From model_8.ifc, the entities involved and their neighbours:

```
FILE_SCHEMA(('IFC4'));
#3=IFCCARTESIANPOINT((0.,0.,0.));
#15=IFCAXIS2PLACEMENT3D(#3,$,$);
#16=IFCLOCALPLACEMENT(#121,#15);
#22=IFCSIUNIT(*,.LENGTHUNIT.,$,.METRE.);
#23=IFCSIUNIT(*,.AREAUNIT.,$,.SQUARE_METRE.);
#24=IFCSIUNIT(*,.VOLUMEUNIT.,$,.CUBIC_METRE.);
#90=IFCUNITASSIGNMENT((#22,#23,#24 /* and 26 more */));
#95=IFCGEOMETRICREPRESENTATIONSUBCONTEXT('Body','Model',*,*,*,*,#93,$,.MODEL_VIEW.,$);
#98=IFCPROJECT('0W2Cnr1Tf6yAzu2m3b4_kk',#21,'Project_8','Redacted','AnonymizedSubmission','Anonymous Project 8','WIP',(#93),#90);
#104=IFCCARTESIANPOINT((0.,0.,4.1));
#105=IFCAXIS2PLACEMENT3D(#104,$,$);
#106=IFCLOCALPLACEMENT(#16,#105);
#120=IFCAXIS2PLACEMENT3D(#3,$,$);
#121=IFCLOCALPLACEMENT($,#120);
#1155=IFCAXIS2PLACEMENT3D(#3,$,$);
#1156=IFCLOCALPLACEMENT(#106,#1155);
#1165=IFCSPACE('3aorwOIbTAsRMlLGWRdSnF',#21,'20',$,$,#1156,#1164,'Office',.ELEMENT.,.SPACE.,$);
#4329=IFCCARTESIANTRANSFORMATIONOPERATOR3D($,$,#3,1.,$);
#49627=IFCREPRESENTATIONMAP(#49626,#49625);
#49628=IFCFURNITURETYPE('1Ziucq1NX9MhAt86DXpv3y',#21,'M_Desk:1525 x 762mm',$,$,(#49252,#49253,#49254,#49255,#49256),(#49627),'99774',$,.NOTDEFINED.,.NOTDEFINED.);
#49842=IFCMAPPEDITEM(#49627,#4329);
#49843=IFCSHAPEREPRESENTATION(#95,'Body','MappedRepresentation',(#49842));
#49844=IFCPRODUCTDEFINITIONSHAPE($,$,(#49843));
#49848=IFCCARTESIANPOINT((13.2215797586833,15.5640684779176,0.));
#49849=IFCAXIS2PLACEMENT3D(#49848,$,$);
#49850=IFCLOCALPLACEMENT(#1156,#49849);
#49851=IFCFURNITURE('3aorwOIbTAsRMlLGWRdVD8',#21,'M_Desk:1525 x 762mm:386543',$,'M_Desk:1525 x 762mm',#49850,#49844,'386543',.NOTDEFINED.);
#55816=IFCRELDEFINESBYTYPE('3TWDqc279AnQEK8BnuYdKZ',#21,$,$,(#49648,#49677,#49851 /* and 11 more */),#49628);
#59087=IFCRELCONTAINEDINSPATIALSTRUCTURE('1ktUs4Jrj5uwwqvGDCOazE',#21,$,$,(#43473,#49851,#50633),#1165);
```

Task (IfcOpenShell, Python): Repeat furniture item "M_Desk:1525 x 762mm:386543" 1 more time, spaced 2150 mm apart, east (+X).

```python
import numpy as np
import ifcopenshell
import ifcopenshell.api.geometry
import ifcopenshell.api.root
import ifcopenshell.util.element
import ifcopenshell.util.placement
import ifcopenshell.util.unit

model = ifcopenshell.open("model_8.ifc")
unit_scale = ifcopenshell.util.unit.calculate_unit_scale(model)


def reuse_history(source, copy):
    """copy_class also copies each property set's owner history, people and application; keep the originals."""
    for rel in copy.IsDefinedBy:
        if rel.is_a("IfcRelDefinesByProperties") and (history := rel.RelatingPropertyDefinition.OwnerHistory):
            rel.RelatingPropertyDefinition.OwnerHistory = source.OwnerHistory
            ifcopenshell.util.element.remove_deep2(model, history)


source = model.by_guid("3aorwOIbTAsRMlLGWRdVD8")
base = ifcopenshell.util.placement.get_local_placement(source.ObjectPlacement)
step = np.array([1.0, 0.0, 0.0]) * 2.15 / unit_scale

for i in range(1, 2):
    copy = ifcopenshell.api.root.copy_class(model, product=source)
    copy.Representation = ifcopenshell.util.element.copy_deep(
        model, source.Representation, exclude=["IfcGeometricRepresentationContext", "IfcRepresentationMap"]
    )
    copy.Name = "M_Desk:1525 x 762mm"
    copy.Tag = None
    reuse_history(source, copy)
    matrix = base.copy()
    matrix[:3, 3] += i * step
    print("added at", matrix[:3, 3].round(3) + 0.0)
    ifcopenshell.api.geometry.edit_object_placement(model, product=copy, matrix=matrix, is_si=False)

model.write("model_8-out.ifc")
```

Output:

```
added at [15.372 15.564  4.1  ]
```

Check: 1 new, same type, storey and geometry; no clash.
